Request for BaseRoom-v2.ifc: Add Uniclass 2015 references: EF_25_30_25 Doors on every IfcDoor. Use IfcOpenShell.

First a look at what the model holds.

```python
import ifcopenshell

model = ifcopenshell.open("BaseRoom-v2.ifc")
print(model.schema)
print("classifications:", [c.Name for c in model.by_type("IfcClassification")])
for ifc_class in ("IfcDoor", "IfcRoof", "IfcStair", "IfcWall", "IfcWindow"):
    print(ifc_class, len(model.by_type(ifc_class)))
```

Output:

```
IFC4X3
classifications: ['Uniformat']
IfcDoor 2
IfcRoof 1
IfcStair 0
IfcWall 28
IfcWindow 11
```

```python
import ifcopenshell
import ifcopenshell.api.classification

model = ifcopenshell.open("BaseRoom-v2.ifc")

system = ifcopenshell.api.classification.add_classification(model, classification="Uniclass 2015")

codes = {
    "IfcDoor": ("EF_25_30_25", "Doors"),
}
for ifc_class, (code, name) in codes.items():
    products = model.by_type(ifc_class)
    ifcopenshell.api.classification.add_reference(
        model, products=products, classification=system, identification=code, name=name
    )
    print(code, len(products))

model.write("BaseRoom-v2-out.ifc")
```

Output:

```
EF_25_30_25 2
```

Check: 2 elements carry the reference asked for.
